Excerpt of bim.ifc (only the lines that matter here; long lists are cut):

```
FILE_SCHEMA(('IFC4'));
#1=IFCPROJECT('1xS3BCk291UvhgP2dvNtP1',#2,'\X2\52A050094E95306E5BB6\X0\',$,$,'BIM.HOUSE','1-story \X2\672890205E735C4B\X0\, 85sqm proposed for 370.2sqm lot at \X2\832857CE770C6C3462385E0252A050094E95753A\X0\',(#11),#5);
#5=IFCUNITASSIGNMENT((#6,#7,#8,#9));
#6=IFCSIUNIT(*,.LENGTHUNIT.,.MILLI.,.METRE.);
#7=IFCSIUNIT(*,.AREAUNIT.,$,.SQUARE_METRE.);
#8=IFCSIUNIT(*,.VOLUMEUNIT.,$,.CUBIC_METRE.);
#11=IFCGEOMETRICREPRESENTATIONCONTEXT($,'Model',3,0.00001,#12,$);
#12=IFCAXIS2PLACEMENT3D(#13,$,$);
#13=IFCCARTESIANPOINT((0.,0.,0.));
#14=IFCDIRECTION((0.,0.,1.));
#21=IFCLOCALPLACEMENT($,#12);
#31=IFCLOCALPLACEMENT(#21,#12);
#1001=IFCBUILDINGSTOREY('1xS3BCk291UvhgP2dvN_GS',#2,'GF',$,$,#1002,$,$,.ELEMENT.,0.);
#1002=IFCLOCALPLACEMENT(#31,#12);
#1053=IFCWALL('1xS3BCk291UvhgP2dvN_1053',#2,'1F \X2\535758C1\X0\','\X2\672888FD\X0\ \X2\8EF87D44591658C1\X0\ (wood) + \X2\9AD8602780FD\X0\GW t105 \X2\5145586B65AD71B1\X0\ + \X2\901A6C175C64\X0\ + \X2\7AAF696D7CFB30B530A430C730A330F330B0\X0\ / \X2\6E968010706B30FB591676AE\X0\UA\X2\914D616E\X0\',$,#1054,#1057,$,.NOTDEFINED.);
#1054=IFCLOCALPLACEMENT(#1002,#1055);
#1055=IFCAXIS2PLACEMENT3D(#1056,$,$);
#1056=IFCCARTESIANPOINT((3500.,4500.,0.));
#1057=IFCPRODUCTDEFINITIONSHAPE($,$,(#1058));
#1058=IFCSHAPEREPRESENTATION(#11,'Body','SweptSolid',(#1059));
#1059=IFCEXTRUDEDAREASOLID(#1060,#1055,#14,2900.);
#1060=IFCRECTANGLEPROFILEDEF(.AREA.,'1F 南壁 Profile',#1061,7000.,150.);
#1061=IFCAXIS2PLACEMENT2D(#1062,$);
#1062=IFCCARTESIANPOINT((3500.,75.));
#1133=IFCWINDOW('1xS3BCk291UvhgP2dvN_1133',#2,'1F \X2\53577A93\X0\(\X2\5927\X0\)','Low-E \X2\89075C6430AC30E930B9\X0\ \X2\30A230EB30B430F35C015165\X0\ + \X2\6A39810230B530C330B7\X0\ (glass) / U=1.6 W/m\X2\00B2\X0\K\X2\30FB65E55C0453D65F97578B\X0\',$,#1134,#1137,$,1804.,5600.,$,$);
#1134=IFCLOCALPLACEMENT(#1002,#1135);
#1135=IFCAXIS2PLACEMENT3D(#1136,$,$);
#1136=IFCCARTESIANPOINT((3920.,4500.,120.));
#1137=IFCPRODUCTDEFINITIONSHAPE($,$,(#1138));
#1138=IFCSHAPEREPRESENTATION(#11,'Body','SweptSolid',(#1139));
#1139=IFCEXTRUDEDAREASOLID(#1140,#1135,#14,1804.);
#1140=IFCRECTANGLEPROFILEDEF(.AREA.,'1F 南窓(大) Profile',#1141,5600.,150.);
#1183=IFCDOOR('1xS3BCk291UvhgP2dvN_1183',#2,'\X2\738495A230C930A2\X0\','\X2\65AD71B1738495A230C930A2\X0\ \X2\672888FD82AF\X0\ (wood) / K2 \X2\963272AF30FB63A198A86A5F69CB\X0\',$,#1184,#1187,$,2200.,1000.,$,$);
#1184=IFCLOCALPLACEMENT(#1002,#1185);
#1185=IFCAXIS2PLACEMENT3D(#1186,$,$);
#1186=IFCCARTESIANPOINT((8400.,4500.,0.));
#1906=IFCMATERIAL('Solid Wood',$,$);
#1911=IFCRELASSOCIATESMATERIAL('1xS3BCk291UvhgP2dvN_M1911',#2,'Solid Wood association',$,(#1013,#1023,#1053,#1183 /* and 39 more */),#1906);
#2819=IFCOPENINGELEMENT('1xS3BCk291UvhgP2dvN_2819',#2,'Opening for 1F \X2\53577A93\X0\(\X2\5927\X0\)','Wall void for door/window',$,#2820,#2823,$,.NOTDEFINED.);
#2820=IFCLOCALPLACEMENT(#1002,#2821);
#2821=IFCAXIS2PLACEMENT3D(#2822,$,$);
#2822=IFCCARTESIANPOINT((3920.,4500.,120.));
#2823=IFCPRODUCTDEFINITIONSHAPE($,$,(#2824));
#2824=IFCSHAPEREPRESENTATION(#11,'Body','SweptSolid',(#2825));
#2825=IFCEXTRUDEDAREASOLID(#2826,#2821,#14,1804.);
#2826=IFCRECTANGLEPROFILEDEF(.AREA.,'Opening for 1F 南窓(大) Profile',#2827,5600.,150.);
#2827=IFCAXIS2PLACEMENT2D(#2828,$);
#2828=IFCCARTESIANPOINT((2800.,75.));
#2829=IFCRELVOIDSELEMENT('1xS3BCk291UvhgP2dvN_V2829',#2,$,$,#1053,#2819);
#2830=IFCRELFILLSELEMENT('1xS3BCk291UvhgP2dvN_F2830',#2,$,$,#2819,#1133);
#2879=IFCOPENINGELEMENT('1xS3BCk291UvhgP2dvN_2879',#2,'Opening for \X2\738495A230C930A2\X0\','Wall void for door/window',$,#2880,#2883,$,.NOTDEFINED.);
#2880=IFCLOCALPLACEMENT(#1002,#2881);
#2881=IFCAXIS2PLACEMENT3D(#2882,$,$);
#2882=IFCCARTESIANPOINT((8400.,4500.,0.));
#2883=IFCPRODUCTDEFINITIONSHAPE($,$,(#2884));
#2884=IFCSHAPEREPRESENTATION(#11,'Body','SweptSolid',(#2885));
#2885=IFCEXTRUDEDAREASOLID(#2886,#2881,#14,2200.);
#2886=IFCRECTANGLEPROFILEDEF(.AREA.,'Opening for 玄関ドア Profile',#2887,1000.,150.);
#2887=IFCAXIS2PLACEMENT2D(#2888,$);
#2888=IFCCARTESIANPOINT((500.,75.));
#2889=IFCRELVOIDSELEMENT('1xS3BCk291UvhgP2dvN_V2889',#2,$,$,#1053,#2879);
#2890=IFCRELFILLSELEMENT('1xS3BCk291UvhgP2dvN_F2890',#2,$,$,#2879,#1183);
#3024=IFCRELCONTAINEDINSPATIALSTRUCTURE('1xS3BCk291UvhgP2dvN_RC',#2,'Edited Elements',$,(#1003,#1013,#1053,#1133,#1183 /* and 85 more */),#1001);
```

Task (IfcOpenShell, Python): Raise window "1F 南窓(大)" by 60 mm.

```python
import numpy as np
import ifcopenshell
import ifcopenshell.api.geometry
import ifcopenshell.util.placement
import ifcopenshell.util.unit

model = ifcopenshell.open("bim.ifc")
unit_scale = ifcopenshell.util.unit.calculate_unit_scale(model)

window = model.by_guid("1xS3BCk291UvhgP2dvN_1133")
opening = window.FillsVoids[0].RelatingOpeningElement
dz = 0.06 / unit_scale

shift = np.array([0.0, 0.0, dz])
# The window is not placed relative to its opening, so move both.
for product in (opening, window):
    matrix = ifcopenshell.util.placement.get_local_placement(product.ObjectPlacement)
    matrix[:3, 3] += shift
    ifcopenshell.api.geometry.edit_object_placement(model, product=product, matrix=matrix, is_si=False)

print(f"moved by {dz * unit_scale:+.3f} m")

model.write("bim_v2.ifc")
```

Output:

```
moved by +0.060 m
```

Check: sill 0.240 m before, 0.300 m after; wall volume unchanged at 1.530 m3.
